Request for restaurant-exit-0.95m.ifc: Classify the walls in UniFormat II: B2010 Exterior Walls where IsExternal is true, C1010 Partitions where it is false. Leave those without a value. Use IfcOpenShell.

First a look at what the model holds.

```python
import ifcopenshell
import ifcopenshell.util.element

model = ifcopenshell.open("restaurant-exit-0.95m.ifc")
print(model.schema)
print("classifications:", [c.Name for c in model.by_type("IfcClassification")])
values = [ifcopenshell.util.element.get_pset(e, "Pset_WallCommon", "IsExternal") for e in model.by_type("IfcWall")]
for value in (True, False, None):
    print("IsExternal", value, values.count(value))
```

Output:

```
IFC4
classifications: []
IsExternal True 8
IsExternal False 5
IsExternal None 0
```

```python
import ifcopenshell
import ifcopenshell.api.classification
import ifcopenshell.util.element

model = ifcopenshell.open("restaurant-exit-0.95m.ifc")

system = ifcopenshell.api.classification.add_classification(model, classification="UniFormat II")

walls = model.by_type("IfcWall")
external = {e: ifcopenshell.util.element.get_pset(e, "Pset_WallCommon", "IsExternal") for e in walls}
for flag, code, name in ((True, "B2010", "Exterior Walls"), (False, "C1010", "Partitions")):
    products = [e for e in walls if external[e] is flag]
    ifcopenshell.api.classification.add_reference(
        model, products=products, classification=system, identification=code, name=name
    )
    print(code, len(products))

model.write("restaurant-exit-0.95m_rev.ifc")
```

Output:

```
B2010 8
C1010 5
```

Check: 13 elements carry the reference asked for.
